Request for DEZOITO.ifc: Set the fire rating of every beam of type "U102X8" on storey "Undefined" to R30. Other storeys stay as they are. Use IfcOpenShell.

First a look at what the model holds.

```python
import ifcopenshell
import ifcopenshell.util.element

model = ifcopenshell.open("DEZOITO.ifc")
print(model.schema)
storey = next(s for s in model.by_type("IfcBuildingStorey") if s.Name == "Undefined")
beams = [e for e in ifcopenshell.util.element.get_decomposition(storey) if e.is_a("IfcBeam")]
seen = {}
for e in beams:
    element_type = ifcopenshell.util.element.get_type(e)
    key = (element_type.Name if element_type != e and element_type else None, ifcopenshell.util.element.get_pset(e, "Pset_BeamCommon", "FireRating"))
    seen[key] = seen.get(key, 0) + 1
for (name, value), count in sorted(seen.items(), key=str):
    print(count, "x", name, "|", value)
```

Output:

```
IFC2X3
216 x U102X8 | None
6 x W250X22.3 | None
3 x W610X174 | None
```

```python
import ifcopenshell
import ifcopenshell.api.pset
import ifcopenshell.util.element

model = ifcopenshell.open("DEZOITO.ifc")

storey = next(s for s in model.by_type("IfcBuildingStorey") if s.Name == "Undefined")
beams = [e for e in ifcopenshell.util.element.get_decomposition(storey) if e.is_a("IfcBeam")]

count = 0
for e in beams:
    element_type = ifcopenshell.util.element.get_type(e)
    if element_type in (None, e) or element_type.Name != "U102X8":
        continue
    found = ifcopenshell.util.element.get_pset(e, "Pset_BeamCommon", should_inherit=False)
    if found:
        pset = model.by_id(found["id"])
        if len(ifcopenshell.util.element.get_elements_by_pset(pset)) > 1:
            pset = ifcopenshell.api.pset.unshare_pset(model, products=[e], pset=pset)[0]
    else:
        pset = ifcopenshell.api.pset.add_pset(model, product=e, name="Pset_BeamCommon")
    ifcopenshell.api.pset.edit_pset(model, pset=pset, properties={"FireRating": "R30"})
    count += 1

print(count, "beams updated")

model.write("DEZOITO_updated.ifc")
```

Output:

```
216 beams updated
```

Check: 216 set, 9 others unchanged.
